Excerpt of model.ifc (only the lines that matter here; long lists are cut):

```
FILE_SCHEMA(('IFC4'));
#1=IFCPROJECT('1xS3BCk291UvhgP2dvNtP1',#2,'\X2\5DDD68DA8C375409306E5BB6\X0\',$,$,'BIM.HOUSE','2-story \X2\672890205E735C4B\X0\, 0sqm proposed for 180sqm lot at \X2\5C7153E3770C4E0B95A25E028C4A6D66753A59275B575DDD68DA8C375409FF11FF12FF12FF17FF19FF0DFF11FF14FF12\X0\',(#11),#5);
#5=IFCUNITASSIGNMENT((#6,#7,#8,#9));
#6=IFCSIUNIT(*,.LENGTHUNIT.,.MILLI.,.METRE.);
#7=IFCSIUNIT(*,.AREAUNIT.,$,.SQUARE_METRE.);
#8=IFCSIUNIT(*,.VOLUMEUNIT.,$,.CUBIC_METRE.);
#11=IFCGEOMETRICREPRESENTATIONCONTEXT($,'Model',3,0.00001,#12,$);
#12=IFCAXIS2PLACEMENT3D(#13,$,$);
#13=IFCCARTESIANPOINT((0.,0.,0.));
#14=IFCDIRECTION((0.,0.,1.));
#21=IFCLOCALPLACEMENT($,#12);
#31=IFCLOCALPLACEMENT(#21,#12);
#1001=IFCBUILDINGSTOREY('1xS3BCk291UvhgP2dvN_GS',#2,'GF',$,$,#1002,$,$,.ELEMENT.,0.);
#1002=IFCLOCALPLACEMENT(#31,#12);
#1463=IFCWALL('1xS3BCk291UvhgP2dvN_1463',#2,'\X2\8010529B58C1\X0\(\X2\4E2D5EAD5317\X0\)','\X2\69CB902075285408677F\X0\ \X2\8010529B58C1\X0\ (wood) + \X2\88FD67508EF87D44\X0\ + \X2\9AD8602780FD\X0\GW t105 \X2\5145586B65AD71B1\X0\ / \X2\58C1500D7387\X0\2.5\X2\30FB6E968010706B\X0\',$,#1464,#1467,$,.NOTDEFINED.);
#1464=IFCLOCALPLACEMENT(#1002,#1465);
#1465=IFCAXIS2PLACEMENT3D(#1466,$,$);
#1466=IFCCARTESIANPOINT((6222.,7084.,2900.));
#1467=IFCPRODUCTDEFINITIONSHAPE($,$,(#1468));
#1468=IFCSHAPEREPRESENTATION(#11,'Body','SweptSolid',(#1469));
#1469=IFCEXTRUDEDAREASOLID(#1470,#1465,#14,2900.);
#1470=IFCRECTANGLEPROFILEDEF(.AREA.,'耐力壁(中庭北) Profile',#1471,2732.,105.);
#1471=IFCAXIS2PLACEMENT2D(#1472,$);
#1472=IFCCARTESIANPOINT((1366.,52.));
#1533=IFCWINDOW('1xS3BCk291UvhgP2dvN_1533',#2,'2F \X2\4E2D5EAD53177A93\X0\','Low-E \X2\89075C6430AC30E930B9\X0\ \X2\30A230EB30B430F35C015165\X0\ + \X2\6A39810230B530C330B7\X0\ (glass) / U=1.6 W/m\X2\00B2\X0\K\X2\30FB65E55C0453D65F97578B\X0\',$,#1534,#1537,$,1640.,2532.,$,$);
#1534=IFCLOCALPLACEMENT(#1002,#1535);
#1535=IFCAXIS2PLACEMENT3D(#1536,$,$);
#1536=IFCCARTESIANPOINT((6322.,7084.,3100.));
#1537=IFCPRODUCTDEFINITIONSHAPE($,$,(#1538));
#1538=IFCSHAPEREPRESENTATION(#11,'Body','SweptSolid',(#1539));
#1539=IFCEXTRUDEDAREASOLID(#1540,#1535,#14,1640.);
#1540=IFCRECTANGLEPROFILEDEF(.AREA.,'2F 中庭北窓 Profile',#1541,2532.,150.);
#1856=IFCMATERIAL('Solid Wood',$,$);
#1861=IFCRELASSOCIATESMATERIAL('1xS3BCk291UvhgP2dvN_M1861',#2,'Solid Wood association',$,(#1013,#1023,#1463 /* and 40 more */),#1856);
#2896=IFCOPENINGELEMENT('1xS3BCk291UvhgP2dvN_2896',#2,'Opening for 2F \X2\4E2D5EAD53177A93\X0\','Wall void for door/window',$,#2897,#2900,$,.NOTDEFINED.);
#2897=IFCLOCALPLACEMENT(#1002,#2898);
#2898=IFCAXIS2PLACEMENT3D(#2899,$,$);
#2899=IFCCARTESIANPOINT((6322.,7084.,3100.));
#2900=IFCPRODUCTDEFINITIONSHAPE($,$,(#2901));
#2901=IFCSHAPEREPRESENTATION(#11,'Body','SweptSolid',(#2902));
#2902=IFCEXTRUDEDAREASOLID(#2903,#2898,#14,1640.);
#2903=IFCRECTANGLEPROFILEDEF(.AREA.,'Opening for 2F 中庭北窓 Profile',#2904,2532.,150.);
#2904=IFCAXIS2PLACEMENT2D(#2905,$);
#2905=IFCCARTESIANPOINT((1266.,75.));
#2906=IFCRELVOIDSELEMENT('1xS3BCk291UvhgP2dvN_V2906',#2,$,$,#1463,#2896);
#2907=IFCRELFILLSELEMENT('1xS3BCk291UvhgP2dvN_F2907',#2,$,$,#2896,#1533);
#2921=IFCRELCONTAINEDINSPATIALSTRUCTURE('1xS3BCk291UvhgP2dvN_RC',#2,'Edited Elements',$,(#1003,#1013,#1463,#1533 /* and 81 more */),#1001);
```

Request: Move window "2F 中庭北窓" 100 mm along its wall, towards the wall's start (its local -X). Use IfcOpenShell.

```python
import ifcopenshell
import ifcopenshell.api.geometry
import ifcopenshell.util.placement
import ifcopenshell.util.unit

model = ifcopenshell.open("model.ifc")
unit_scale = ifcopenshell.util.unit.calculate_unit_scale(model)

window = model.by_id(1533)
opening = window.FillsVoids[0].RelatingOpeningElement
wall = opening.VoidsElements[0].RelatingBuildingElement

wall_matrix = ifcopenshell.util.placement.get_local_placement(wall.ObjectPlacement)
shift = wall_matrix[:3, 0] * -0.1 / unit_scale
before = ifcopenshell.util.placement.get_local_placement(window.ObjectPlacement)[:3, 3].copy()

# The window is not placed relative to its opening, so move both.
for product in (opening, window):
    matrix = ifcopenshell.util.placement.get_local_placement(product.ObjectPlacement)
    matrix[:3, 3] += shift
    ifcopenshell.api.geometry.edit_object_placement(model, product=product, matrix=matrix, is_si=False)

after = ifcopenshell.util.placement.get_local_placement(window.ObjectPlacement)[:3, 3]
print("window moved by", (after - before).round(3) + 0.0)

model.write("model_edited.ifc")
```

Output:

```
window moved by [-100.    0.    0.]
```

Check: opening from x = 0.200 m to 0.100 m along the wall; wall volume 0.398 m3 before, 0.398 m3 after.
